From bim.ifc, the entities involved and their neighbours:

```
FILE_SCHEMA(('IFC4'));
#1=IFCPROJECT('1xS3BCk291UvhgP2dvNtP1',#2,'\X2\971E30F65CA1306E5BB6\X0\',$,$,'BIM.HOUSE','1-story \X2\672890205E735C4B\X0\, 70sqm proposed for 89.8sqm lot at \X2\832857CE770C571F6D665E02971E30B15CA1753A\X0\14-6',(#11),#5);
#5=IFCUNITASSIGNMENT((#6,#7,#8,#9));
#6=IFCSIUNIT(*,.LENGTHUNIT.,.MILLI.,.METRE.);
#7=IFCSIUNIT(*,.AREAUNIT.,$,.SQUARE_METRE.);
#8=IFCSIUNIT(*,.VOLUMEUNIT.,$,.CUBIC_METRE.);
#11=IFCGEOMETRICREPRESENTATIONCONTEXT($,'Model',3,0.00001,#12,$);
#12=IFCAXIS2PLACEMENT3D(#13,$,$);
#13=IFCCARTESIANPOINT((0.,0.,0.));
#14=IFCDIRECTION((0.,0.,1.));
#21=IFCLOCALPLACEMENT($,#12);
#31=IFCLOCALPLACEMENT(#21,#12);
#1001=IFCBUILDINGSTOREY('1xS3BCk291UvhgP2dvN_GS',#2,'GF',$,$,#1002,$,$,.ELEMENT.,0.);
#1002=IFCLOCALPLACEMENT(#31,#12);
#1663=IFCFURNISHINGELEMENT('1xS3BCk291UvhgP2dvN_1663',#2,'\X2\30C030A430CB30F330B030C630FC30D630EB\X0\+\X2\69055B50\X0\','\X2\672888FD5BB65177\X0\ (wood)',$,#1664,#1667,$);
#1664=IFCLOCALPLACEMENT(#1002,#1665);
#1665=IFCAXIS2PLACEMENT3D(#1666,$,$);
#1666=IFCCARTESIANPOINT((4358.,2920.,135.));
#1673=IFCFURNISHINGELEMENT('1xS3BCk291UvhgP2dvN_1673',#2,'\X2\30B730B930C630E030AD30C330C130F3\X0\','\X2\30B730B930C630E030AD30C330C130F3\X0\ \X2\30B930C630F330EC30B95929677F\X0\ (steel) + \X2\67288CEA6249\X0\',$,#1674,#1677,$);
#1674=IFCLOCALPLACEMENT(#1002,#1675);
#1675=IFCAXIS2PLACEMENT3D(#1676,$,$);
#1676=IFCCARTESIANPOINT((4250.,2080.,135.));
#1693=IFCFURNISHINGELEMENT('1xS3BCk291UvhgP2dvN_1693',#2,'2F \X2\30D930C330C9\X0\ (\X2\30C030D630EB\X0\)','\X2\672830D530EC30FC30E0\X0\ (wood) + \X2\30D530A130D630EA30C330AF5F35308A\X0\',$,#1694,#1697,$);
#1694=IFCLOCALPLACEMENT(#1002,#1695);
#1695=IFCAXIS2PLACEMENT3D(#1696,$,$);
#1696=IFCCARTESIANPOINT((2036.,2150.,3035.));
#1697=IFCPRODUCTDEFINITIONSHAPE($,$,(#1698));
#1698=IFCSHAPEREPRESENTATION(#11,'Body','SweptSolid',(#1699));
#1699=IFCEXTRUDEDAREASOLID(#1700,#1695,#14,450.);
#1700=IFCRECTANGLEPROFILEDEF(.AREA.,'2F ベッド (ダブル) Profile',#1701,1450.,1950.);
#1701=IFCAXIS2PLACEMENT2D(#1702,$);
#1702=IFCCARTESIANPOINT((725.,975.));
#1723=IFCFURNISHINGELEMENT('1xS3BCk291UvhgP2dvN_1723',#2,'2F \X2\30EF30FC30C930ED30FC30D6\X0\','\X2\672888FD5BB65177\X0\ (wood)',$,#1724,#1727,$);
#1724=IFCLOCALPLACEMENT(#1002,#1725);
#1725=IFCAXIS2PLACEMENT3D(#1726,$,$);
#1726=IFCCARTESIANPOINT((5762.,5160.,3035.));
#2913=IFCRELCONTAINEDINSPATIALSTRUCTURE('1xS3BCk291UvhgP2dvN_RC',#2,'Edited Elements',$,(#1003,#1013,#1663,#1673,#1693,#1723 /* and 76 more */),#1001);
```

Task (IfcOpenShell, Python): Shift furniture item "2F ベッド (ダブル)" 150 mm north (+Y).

```python
import ifcopenshell
import ifcopenshell.api.geometry
import ifcopenshell.util.placement
import ifcopenshell.util.unit

model = ifcopenshell.open("bim.ifc")
unit_scale = ifcopenshell.util.unit.calculate_unit_scale(model)

item = model.by_guid("1xS3BCk291UvhgP2dvN_1693")
matrix = ifcopenshell.util.placement.get_local_placement(item.ObjectPlacement)
matrix[1, 3] += 0.15 / unit_scale
ifcopenshell.api.geometry.edit_object_placement(model, product=item, matrix=matrix, is_si=False)

print(ifcopenshell.util.placement.get_local_placement(item.ObjectPlacement).round(3) + 0.0)

model.write("bim_v2.ifc")
```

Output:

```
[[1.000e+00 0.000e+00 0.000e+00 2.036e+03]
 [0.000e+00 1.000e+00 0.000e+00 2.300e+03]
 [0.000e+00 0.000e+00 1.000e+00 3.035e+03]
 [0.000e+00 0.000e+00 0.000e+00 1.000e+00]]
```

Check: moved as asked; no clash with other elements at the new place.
